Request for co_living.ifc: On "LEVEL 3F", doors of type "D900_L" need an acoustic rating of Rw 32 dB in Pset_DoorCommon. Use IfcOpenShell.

First a look at what the model holds.

```python
import ifcopenshell
import ifcopenshell.util.element

model = ifcopenshell.open("co_living.ifc")
print(model.schema)
storey = next(s for s in model.by_type("IfcBuildingStorey") if s.Name == "LEVEL 3F")
doors = [e for e in ifcopenshell.util.element.get_decomposition(storey) if e.is_a("IfcDoor")]
seen = {}
for e in doors:
    element_type = ifcopenshell.util.element.get_type(e)
    key = (element_type.Name if element_type != e and element_type else None, ifcopenshell.util.element.get_pset(e, "Pset_DoorCommon", "AcousticRating"))
    seen[key] = seen.get(key, 0) + 1
for (name, value), count in sorted(seen.items(), key=str):
    print(count, "x", name, "|", value)
```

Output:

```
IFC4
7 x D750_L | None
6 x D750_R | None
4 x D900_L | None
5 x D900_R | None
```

```python
import ifcopenshell
import ifcopenshell.api.pset
import ifcopenshell.util.element

model = ifcopenshell.open("co_living.ifc")

storey = next(s for s in model.by_type("IfcBuildingStorey") if s.Name == "LEVEL 3F")
doors = [e for e in ifcopenshell.util.element.get_decomposition(storey) if e.is_a("IfcDoor")]

count = 0
for e in doors:
    element_type = ifcopenshell.util.element.get_type(e)
    if element_type in (None, e) or element_type.Name != "D900_L":
        continue
    # add_pset returns the element's existing set when there is one.
    pset = ifcopenshell.api.pset.add_pset(model, product=e, name="Pset_DoorCommon")
    ifcopenshell.api.pset.edit_pset(model, pset=pset, properties={"AcousticRating": "Rw 32 dB"})
    count += 1

print(count, "doors updated")

model.write("co_living-out.ifc")
```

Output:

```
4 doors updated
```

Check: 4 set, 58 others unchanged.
